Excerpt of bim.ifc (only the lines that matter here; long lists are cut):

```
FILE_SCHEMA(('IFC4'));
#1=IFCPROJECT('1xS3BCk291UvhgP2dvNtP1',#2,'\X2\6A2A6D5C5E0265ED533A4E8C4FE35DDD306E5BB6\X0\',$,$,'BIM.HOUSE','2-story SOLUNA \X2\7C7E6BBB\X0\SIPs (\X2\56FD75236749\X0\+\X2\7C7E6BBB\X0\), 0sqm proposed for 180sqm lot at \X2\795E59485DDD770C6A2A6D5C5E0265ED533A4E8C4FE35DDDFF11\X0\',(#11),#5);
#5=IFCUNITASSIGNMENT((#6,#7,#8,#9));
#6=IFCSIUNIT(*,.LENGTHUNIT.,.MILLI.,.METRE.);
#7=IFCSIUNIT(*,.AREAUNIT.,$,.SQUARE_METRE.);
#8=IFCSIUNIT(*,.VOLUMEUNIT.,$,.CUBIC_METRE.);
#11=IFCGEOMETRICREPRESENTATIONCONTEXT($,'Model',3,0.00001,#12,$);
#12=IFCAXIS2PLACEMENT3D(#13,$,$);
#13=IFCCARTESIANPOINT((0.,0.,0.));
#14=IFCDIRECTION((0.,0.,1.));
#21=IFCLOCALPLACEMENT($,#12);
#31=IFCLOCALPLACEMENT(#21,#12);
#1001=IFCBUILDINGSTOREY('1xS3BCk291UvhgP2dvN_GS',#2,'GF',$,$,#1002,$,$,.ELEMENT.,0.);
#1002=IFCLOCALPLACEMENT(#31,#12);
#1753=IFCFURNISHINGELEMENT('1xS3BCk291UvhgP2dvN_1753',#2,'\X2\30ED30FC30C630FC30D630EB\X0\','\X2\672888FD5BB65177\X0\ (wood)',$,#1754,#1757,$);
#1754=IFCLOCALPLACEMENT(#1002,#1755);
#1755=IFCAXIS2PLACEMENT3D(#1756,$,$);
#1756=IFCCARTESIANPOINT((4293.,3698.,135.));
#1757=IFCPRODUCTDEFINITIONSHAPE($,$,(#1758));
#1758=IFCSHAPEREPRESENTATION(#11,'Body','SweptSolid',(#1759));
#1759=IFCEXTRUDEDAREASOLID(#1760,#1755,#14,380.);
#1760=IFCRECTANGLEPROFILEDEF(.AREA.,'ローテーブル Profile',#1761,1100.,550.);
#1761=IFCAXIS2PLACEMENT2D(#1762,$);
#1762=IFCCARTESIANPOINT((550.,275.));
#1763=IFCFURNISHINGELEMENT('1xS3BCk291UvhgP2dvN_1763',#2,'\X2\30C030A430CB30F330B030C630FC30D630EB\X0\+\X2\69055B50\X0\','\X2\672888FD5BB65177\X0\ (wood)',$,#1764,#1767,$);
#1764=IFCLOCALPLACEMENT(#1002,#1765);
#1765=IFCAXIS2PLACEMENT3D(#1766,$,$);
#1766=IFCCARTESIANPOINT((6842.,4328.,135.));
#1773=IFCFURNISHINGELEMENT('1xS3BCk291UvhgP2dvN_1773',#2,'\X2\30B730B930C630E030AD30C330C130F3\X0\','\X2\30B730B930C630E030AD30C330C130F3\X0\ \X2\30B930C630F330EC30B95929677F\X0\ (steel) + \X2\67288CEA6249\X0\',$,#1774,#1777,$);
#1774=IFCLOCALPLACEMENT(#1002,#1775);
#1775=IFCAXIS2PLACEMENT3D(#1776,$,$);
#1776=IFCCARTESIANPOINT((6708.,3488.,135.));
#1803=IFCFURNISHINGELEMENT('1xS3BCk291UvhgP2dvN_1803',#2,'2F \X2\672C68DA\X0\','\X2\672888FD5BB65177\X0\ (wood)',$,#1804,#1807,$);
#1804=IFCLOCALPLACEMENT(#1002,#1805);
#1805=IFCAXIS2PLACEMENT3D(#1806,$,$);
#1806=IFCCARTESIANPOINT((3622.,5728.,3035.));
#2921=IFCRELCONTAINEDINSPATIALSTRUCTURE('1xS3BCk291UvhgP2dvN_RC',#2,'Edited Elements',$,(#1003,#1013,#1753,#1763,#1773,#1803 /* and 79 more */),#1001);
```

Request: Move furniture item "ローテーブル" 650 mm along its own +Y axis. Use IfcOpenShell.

```python
import ifcopenshell
import ifcopenshell.api.geometry
import ifcopenshell.util.placement
import ifcopenshell.util.unit

model = ifcopenshell.open("bim.ifc")
unit_scale = ifcopenshell.util.unit.calculate_unit_scale(model)

item = model.by_guid("1xS3BCk291UvhgP2dvN_1753")
matrix = ifcopenshell.util.placement.get_local_placement(item.ObjectPlacement)
matrix[:3, 3] += matrix[:3, 1] * 0.65 / unit_scale
ifcopenshell.api.geometry.edit_object_placement(model, product=item, matrix=matrix, is_si=False)

print(ifcopenshell.util.placement.get_local_placement(item.ObjectPlacement).round(3) + 0.0)

model.write("bim_v2.ifc")
```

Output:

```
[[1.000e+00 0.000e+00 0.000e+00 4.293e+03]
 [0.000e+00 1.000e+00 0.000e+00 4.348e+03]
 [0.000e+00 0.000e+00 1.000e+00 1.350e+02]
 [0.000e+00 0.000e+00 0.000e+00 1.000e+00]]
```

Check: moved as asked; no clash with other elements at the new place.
